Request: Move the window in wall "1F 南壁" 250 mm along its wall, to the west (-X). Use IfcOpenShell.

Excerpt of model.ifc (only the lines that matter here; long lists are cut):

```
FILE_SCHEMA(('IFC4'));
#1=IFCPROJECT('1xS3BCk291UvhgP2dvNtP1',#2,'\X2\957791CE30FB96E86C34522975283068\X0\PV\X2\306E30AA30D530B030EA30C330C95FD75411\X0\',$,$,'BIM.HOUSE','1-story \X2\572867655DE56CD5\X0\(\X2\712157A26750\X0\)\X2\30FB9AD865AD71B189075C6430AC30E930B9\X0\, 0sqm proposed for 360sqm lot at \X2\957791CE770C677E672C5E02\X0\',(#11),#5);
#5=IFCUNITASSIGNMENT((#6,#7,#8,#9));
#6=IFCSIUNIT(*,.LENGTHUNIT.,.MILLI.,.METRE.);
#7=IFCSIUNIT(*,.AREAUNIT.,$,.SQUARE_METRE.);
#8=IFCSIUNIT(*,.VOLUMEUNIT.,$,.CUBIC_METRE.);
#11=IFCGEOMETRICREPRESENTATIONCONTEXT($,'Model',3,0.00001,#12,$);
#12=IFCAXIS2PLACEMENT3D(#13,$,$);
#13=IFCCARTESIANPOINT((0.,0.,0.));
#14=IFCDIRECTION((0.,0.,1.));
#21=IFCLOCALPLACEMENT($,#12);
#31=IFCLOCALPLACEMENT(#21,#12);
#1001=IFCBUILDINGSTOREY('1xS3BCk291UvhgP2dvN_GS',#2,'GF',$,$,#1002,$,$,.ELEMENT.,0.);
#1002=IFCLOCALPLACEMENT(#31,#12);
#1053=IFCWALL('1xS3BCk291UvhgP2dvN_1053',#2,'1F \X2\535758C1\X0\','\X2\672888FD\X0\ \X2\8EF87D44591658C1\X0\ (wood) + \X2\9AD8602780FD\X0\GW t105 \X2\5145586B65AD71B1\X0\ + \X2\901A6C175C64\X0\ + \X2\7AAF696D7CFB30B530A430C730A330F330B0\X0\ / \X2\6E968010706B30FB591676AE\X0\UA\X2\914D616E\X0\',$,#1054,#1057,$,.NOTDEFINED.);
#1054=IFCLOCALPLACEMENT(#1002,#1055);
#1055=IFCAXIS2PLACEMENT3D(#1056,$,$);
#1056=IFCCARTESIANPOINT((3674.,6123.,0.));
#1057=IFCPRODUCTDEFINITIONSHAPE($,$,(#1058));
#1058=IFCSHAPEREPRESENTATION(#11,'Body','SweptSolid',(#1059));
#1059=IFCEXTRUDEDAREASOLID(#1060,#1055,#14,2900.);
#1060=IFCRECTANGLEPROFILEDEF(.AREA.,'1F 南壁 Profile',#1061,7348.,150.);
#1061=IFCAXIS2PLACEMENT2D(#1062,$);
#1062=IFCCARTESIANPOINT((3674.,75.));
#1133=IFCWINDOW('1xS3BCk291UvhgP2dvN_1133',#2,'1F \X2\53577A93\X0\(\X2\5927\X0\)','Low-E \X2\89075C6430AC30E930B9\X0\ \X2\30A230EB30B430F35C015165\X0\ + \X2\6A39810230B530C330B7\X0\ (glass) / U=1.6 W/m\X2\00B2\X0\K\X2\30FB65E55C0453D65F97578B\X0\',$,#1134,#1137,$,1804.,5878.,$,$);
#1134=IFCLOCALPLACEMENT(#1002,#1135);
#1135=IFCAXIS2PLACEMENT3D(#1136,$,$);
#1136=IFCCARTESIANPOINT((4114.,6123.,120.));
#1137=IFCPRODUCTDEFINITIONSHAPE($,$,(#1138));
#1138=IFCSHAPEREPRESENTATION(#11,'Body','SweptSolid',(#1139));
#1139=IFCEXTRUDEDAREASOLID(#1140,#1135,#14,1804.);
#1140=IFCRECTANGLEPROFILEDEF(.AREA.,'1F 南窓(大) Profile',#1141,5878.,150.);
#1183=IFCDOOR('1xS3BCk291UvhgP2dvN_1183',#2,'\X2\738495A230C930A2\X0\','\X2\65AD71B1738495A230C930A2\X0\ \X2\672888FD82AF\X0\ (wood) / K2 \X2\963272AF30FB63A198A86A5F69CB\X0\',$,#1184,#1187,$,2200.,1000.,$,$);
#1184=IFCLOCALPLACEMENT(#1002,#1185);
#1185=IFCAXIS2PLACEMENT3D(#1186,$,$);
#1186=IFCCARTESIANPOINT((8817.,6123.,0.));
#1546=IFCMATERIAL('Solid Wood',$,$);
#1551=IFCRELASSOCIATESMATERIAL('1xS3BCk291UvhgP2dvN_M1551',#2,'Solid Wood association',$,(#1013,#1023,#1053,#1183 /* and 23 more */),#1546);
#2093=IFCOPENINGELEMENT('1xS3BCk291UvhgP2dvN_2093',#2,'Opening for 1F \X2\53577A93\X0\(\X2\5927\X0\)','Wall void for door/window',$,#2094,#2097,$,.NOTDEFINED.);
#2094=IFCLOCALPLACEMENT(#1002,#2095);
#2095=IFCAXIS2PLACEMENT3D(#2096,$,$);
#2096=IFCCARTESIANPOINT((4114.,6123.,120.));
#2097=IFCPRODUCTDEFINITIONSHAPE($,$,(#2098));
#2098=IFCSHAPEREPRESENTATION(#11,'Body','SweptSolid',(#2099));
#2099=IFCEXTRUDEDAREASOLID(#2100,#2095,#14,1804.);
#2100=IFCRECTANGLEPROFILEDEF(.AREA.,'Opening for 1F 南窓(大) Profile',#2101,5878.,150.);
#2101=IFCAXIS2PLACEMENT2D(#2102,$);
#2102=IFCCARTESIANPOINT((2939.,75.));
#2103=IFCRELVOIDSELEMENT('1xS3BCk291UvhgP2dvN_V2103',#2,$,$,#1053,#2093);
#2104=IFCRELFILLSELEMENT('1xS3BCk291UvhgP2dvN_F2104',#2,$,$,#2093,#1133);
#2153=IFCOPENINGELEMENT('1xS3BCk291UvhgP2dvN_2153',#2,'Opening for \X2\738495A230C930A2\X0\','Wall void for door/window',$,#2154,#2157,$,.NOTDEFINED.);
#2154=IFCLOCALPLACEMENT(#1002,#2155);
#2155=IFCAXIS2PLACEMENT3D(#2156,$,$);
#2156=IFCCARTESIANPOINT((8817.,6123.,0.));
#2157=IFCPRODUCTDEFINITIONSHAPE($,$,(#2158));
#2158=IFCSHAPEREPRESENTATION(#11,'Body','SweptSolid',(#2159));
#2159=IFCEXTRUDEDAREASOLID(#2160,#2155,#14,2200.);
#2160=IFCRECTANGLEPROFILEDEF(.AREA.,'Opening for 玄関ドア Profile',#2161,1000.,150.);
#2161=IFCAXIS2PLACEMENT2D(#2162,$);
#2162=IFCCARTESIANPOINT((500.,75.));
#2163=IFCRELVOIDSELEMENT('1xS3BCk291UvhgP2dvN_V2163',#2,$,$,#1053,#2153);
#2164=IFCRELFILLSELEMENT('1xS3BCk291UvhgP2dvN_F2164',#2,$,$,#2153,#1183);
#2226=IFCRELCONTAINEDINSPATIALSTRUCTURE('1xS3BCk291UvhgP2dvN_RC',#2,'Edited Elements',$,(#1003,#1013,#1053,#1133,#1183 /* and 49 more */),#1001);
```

```python
import ifcopenshell
import ifcopenshell.api.geometry
import ifcopenshell.util.placement
import ifcopenshell.util.unit

model = ifcopenshell.open("model.ifc")
unit_scale = ifcopenshell.util.unit.calculate_unit_scale(model)

window = model.by_guid("1xS3BCk291UvhgP2dvN_1133")
opening = window.FillsVoids[0].RelatingOpeningElement
wall = opening.VoidsElements[0].RelatingBuildingElement

wall_matrix = ifcopenshell.util.placement.get_local_placement(wall.ObjectPlacement)
shift = wall_matrix[:3, 0] * -0.25 / unit_scale
before = ifcopenshell.util.placement.get_local_placement(window.ObjectPlacement)[:3, 3].copy()

# The window is not placed relative to its opening, so move both.
for product in (opening, window):
    matrix = ifcopenshell.util.placement.get_local_placement(product.ObjectPlacement)
    matrix[:3, 3] += shift
    ifcopenshell.api.geometry.edit_object_placement(model, product=product, matrix=matrix, is_si=False)

after = ifcopenshell.util.placement.get_local_placement(window.ObjectPlacement)[:3, 3]
print("window moved by", (after - before).round(3) + 0.0)

model.write("model_updated.ifc")
```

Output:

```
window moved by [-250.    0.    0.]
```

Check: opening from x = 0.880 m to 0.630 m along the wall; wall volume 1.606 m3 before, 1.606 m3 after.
